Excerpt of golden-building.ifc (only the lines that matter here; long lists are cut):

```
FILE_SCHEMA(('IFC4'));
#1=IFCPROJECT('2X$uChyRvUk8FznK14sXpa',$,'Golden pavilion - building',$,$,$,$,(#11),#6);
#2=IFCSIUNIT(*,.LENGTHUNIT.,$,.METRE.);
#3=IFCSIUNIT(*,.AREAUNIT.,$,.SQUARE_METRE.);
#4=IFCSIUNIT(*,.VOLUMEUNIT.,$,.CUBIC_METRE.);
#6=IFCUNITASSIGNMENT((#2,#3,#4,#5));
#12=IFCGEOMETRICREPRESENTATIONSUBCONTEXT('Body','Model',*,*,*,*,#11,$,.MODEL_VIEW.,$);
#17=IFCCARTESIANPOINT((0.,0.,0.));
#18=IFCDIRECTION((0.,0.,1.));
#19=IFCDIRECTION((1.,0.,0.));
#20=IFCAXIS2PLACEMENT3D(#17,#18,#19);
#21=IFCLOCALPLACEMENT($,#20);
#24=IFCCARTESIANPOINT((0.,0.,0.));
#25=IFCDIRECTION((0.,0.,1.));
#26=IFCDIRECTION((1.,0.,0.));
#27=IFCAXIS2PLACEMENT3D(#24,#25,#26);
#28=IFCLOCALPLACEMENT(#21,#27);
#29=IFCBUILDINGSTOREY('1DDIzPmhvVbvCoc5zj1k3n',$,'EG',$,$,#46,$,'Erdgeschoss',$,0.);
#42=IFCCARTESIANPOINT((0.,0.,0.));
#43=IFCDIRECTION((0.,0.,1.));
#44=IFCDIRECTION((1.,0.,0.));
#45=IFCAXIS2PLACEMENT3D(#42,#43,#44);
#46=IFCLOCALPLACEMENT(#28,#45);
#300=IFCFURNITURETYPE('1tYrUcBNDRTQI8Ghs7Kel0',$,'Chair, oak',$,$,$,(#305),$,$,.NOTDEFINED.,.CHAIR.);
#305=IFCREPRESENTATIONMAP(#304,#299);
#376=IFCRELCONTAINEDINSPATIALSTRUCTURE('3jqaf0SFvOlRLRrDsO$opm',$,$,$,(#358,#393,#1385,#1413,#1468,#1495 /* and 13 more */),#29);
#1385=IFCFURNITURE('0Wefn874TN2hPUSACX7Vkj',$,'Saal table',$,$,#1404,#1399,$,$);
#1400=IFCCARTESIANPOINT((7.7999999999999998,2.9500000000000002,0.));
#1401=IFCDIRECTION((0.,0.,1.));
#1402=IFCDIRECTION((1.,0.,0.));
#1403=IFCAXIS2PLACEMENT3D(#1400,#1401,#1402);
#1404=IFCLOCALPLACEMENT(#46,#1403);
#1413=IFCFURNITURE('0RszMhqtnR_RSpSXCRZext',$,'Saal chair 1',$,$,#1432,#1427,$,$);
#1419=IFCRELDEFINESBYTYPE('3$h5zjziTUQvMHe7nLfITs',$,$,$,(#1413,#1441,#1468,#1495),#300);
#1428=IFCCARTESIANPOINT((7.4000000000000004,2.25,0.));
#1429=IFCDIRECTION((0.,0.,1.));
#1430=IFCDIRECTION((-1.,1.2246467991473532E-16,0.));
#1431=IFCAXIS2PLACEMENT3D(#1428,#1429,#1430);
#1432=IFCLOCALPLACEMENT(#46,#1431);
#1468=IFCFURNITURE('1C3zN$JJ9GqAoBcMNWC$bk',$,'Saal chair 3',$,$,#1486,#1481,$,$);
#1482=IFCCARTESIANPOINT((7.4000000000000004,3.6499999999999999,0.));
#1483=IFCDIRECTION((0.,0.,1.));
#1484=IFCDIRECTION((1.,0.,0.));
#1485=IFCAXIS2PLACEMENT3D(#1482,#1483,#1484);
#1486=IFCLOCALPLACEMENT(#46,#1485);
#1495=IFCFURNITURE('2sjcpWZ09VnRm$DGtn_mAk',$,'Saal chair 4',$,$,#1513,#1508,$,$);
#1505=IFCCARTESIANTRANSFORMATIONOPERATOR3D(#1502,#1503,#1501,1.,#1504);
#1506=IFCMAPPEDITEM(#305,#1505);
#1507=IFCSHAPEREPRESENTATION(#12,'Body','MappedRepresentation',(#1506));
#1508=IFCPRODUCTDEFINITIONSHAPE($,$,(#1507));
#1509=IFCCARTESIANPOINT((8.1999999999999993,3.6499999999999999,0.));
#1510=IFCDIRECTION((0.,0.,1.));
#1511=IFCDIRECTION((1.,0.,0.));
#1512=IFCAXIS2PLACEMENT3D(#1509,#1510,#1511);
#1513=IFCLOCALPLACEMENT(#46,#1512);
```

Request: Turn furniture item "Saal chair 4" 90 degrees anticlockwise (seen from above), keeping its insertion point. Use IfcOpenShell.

```python
import ifcopenshell
import ifcopenshell.api.geometry
import ifcopenshell.util.placement

model = ifcopenshell.open("golden-building.ifc")

item = model.by_guid("2sjcpWZ09VnRm$DGtn_mAk")
matrix = ifcopenshell.util.placement.get_local_placement(item.ObjectPlacement)
matrix = matrix @ ifcopenshell.util.placement.rotation(90, "Z")
ifcopenshell.api.geometry.edit_object_placement(model, product=item, matrix=matrix, is_si=False)

print(ifcopenshell.util.placement.get_local_placement(item.ObjectPlacement).round(3) + 0.0)

model.write("golden-building_rev.ifc")
```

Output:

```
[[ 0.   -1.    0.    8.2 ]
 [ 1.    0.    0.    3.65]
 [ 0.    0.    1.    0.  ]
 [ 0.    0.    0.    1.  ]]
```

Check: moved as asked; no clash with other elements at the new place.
